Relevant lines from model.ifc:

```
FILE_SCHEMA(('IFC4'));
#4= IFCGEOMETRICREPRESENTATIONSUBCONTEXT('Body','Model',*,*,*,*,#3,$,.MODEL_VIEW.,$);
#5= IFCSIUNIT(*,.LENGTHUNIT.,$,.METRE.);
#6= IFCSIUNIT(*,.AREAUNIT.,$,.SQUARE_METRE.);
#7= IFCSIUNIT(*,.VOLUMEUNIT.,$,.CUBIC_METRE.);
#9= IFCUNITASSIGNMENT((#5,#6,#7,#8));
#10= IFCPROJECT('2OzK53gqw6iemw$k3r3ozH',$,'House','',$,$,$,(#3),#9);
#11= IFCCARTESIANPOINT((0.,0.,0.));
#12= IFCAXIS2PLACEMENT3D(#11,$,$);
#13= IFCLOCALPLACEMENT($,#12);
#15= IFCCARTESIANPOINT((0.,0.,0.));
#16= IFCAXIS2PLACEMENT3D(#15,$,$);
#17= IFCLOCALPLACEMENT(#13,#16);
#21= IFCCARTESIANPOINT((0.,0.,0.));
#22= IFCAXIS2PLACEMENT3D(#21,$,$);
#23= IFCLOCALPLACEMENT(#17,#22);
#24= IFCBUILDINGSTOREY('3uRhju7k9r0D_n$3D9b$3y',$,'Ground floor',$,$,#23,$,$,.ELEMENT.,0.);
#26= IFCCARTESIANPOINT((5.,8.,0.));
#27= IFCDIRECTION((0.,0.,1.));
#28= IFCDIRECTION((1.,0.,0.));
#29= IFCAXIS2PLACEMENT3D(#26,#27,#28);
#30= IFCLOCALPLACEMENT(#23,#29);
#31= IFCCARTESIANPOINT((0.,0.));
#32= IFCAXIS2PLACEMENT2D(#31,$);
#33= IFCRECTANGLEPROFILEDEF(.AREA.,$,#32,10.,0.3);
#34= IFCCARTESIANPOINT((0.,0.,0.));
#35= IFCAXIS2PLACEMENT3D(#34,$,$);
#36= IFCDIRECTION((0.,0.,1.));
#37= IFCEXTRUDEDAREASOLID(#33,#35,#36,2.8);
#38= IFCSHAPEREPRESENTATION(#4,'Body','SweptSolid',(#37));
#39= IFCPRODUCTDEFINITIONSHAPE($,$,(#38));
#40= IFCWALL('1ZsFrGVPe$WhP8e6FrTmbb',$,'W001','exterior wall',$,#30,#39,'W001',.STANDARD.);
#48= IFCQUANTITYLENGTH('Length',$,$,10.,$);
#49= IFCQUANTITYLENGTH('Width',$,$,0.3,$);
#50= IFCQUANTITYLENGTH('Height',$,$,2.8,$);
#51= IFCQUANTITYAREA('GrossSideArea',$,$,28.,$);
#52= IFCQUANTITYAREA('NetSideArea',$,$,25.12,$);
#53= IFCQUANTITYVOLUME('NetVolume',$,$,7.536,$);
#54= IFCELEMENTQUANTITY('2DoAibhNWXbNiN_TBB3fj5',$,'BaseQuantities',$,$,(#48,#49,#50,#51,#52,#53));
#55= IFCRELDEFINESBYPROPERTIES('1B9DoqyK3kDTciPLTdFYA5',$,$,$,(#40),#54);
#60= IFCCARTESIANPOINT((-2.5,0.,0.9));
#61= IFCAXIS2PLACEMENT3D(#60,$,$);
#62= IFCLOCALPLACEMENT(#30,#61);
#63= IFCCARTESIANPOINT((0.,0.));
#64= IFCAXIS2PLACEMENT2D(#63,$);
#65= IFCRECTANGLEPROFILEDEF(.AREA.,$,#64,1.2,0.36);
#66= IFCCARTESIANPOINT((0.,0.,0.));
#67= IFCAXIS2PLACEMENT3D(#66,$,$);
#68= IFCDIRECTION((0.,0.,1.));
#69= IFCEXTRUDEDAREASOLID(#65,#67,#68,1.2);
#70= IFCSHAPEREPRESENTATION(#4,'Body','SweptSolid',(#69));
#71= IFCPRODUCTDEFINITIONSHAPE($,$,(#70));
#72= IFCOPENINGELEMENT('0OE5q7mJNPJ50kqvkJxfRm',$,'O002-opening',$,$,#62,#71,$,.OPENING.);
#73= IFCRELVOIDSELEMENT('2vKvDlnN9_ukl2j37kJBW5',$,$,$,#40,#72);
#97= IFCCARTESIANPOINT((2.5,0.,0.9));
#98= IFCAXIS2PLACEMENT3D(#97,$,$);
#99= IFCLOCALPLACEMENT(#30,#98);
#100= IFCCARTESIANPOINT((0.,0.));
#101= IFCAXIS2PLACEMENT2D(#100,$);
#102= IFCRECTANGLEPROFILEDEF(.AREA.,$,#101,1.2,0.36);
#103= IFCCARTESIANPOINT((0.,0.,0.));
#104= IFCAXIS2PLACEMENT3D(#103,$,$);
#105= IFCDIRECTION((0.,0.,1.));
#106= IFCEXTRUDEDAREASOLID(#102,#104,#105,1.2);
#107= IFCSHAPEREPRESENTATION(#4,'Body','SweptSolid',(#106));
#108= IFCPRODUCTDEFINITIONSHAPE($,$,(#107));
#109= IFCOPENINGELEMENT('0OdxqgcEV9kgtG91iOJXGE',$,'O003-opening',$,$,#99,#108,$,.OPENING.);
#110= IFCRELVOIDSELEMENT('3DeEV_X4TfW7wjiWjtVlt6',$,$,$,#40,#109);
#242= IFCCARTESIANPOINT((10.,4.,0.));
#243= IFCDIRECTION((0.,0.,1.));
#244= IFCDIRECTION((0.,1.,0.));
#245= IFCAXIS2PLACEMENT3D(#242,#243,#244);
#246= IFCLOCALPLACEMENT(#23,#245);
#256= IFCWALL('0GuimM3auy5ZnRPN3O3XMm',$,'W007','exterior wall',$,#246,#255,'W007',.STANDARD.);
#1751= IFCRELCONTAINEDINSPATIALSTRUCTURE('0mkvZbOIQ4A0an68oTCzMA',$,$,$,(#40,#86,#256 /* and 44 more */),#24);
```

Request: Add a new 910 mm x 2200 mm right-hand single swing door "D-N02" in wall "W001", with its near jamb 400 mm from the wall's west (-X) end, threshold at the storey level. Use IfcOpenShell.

```python
import numpy as np
import ifcopenshell
import ifcopenshell.api.feature
import ifcopenshell.api.geometry
import ifcopenshell.api.pset
import ifcopenshell.api.root
import ifcopenshell.api.spatial
import ifcopenshell.geom
import ifcopenshell.util.element
import ifcopenshell.util.placement
import ifcopenshell.util.representation
import ifcopenshell.util.shape
import ifcopenshell.util.unit

model = ifcopenshell.open("model.ifc")
unit_scale = ifcopenshell.util.unit.calculate_unit_scale(model)
area_scale = ifcopenshell.util.unit.calculate_unit_scale(model, "AREAUNIT")
volume_scale = ifcopenshell.util.unit.calculate_unit_scale(model, "VOLUMEUNIT")
settings = ifcopenshell.geom.settings()


def volume(element):
    """Net volume in cubic metres, openings subtracted."""
    shape = ifcopenshell.geom.create_shape(settings, element)
    return ifcopenshell.util.shape.get_volume(shape.geometry)


wall = model.by_id(40)
storey = ifcopenshell.util.element.get_container(wall, ifc_class="IfcBuildingStorey")
context = ifcopenshell.util.representation.get_context(model, "Model", "Body", "MODEL_VIEW")
before = volume(wall)

width, height, from_end, sill = 0.91, 2.2, 0.4, 0.0  # metres

# The wall runs along its own X axis, and the end named is its -X end.
wall_shape = ifcopenshell.geom.create_shape(settings, wall)
x, y, z = ifcopenshell.util.shape.get_vertices(wall_shape.geometry).T
start = x.min() + from_end
face, thickness = float(y.min()), float(y.max() - y.min())
wall_matrix = ifcopenshell.util.placement.get_local_placement(wall.ObjectPlacement)
level = ifcopenshell.util.placement.get_local_placement(storey.ObjectPlacement)[2, 3]


def in_wall(x, y):
    """Placement at x, y metres in the wall's axes, at sill height."""
    matrix = wall_matrix.copy()
    matrix[:, 3] = wall_matrix @ np.array([x / unit_scale, y / unit_scale, 0.0, 1.0])
    matrix[2, 3] = level + sill / unit_scale
    return matrix


# Opening: a box that overshoots both wall faces by 50 mm.
opening = ifcopenshell.api.root.create_entity(model, ifc_class="IfcOpeningElement", predefined_type="OPENING")
box = ifcopenshell.api.geometry.add_wall_representation(
    model, context=context, length=width, height=height, thickness=thickness + 0.1
)
ifcopenshell.api.geometry.assign_representation(model, product=opening, representation=box)
ifcopenshell.api.geometry.edit_object_placement(model, product=opening, matrix=in_wall(start, face - 0.05), is_si=False)
ifcopenshell.api.feature.add_feature(model, feature=opening, element=wall)

door = ifcopenshell.api.root.create_entity(model, ifc_class="IfcDoor", name="D-N02", predefined_type="DOOR")
door.OverallWidth, door.OverallHeight = width / unit_scale, height / unit_scale
door.OperationType = "SINGLE_SWING_RIGHT"
body = ifcopenshell.api.geometry.add_door_representation(
    model,
    context=context,
    overall_width=door.OverallWidth,
    overall_height=door.OverallHeight,
    operation_type="SINGLE_SWING_RIGHT",
    lining_properties={"LiningDepth": thickness / unit_scale, "ThresholdDepth": thickness / unit_scale},
)
ifcopenshell.api.geometry.assign_representation(model, product=door, representation=body)
ifcopenshell.api.spatial.assign_container(model, products=[door], relating_structure=storey)
ifcopenshell.api.feature.add_filling(model, opening=opening, element=door)

# The lining spans the wall, so the door starts at the wall face.
ifcopenshell.api.geometry.edit_object_placement(model, product=door, matrix=in_wall(start, face), is_si=False)

after = volume(wall)

# Update the wall's stored quantities.
qto = model.by_id(ifcopenshell.util.element.get_pset(wall, "BaseQuantities", should_inherit=False)["id"])
ifcopenshell.api.pset.edit_qto(model, qto=qto, properties={
    "NetSideArea": after / thickness / area_scale,
    "NetVolume": after / volume_scale,
})

print(f"wall volume {before:.3f} -> {after:.3f} m3")

model.write("model-out.ifc")
```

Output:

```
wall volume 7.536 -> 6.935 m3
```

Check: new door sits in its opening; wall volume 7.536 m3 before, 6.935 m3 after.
